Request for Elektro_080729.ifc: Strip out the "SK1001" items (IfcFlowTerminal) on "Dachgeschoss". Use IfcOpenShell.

First a look at what the model holds.

```python
import ifcopenshell
import ifcopenshell.util.element

model = ifcopenshell.open("Elektro_080729.ifc")
print(model.schema)
storey = next(s for s in model.by_type("IfcBuildingStorey") if s.Name == "Dachgeschoss")
terminals = [e for e in ifcopenshell.util.element.get_decomposition(storey) if e.is_a("IfcFlowTerminal")]
seen = {}
for e in terminals:
    element_type = ifcopenshell.util.element.get_type(e)
    name = element_type.Name if element_type not in (None, e) else None
    seen[name] = seen.get(name, 0) + 1
for name, count in sorted(seen.items(), key=str):
    print(count, "x", name)
```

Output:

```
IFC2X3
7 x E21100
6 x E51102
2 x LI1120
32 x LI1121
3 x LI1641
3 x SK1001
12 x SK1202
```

```python
import ifcopenshell
import ifcopenshell.api.root
import ifcopenshell.util.element

model = ifcopenshell.open("Elektro_080729.ifc")

storey = next(s for s in model.by_type("IfcBuildingStorey") if s.Name == "Dachgeschoss")
terminals = [e for e in ifcopenshell.util.element.get_decomposition(storey) if e.is_a("IfcFlowTerminal")]
targets = [e for e in terminals if (t := ifcopenshell.util.element.get_type(e)) not in (None, e) and t.Name == "SK1001"]

for e in targets:
    ifcopenshell.api.root.remove_product(model, product=e)
print(len(targets), "removed")

model.write("Elektro_080729_edited.ifc")
```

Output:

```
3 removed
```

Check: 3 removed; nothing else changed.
